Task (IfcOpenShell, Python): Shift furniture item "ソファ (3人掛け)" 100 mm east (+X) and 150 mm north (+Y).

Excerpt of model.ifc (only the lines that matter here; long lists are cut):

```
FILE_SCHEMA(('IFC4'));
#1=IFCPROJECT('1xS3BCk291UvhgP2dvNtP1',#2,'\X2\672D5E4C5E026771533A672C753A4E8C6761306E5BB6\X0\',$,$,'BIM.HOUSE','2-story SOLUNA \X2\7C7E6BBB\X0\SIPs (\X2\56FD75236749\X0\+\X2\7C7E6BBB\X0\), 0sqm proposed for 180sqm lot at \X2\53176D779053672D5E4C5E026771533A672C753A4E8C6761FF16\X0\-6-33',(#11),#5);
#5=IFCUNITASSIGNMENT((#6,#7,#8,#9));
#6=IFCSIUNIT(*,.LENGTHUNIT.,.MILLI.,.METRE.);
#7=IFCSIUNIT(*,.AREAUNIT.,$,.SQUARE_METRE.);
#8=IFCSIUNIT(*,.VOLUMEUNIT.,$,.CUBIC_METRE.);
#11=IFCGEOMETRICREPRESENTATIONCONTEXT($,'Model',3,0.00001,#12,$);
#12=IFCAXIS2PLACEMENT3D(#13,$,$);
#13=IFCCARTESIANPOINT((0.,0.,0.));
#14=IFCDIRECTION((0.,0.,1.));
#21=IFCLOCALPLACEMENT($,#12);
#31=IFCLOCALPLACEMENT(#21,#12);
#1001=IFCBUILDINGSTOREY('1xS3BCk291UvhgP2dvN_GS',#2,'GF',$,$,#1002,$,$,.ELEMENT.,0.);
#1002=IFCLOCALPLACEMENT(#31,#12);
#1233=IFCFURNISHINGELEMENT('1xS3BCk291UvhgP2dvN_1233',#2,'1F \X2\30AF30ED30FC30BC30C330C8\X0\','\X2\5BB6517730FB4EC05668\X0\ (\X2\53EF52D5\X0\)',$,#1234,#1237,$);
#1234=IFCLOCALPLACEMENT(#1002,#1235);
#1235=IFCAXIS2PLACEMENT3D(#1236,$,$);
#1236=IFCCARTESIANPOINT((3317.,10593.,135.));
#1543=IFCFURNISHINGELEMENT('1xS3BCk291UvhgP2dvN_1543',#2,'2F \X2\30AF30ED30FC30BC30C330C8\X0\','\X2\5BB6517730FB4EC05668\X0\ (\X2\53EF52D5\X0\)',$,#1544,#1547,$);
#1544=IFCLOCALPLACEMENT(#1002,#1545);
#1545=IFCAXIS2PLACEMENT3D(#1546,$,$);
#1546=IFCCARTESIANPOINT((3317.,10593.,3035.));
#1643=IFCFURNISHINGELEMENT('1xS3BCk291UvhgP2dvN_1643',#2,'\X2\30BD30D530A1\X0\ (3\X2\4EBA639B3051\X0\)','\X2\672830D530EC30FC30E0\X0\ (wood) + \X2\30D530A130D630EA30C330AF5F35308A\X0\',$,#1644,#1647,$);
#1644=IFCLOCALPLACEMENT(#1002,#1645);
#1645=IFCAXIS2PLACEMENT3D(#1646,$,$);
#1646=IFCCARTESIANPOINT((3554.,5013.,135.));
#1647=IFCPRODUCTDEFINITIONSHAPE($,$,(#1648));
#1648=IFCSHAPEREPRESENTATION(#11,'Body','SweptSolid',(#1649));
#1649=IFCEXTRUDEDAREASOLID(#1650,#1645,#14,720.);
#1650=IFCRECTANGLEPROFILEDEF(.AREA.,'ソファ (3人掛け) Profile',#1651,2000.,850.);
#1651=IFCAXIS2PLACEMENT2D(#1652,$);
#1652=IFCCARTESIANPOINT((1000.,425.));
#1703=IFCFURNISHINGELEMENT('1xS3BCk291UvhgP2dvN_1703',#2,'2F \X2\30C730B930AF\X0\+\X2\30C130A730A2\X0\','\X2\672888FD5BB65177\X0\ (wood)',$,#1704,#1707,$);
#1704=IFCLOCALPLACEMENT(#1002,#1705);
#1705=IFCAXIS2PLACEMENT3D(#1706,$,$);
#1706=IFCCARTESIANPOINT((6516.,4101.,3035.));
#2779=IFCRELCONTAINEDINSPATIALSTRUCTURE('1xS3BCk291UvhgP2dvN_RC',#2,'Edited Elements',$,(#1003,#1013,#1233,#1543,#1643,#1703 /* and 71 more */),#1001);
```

```python
import ifcopenshell
import ifcopenshell.api.geometry
import ifcopenshell.util.placement
import ifcopenshell.util.unit

model = ifcopenshell.open("model.ifc")
unit_scale = ifcopenshell.util.unit.calculate_unit_scale(model)

item = model.by_guid("1xS3BCk291UvhgP2dvN_1643")
matrix = ifcopenshell.util.placement.get_local_placement(item.ObjectPlacement)
matrix[0, 3] += 0.1 / unit_scale
matrix[1, 3] += 0.15 / unit_scale
ifcopenshell.api.geometry.edit_object_placement(model, product=item, matrix=matrix, is_si=False)

print(ifcopenshell.util.placement.get_local_placement(item.ObjectPlacement).round(3) + 0.0)

model.write("model_updated.ifc")
```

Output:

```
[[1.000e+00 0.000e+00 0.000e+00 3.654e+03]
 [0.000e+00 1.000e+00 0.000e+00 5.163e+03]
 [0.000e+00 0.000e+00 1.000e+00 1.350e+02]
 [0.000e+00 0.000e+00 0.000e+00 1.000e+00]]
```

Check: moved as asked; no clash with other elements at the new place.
